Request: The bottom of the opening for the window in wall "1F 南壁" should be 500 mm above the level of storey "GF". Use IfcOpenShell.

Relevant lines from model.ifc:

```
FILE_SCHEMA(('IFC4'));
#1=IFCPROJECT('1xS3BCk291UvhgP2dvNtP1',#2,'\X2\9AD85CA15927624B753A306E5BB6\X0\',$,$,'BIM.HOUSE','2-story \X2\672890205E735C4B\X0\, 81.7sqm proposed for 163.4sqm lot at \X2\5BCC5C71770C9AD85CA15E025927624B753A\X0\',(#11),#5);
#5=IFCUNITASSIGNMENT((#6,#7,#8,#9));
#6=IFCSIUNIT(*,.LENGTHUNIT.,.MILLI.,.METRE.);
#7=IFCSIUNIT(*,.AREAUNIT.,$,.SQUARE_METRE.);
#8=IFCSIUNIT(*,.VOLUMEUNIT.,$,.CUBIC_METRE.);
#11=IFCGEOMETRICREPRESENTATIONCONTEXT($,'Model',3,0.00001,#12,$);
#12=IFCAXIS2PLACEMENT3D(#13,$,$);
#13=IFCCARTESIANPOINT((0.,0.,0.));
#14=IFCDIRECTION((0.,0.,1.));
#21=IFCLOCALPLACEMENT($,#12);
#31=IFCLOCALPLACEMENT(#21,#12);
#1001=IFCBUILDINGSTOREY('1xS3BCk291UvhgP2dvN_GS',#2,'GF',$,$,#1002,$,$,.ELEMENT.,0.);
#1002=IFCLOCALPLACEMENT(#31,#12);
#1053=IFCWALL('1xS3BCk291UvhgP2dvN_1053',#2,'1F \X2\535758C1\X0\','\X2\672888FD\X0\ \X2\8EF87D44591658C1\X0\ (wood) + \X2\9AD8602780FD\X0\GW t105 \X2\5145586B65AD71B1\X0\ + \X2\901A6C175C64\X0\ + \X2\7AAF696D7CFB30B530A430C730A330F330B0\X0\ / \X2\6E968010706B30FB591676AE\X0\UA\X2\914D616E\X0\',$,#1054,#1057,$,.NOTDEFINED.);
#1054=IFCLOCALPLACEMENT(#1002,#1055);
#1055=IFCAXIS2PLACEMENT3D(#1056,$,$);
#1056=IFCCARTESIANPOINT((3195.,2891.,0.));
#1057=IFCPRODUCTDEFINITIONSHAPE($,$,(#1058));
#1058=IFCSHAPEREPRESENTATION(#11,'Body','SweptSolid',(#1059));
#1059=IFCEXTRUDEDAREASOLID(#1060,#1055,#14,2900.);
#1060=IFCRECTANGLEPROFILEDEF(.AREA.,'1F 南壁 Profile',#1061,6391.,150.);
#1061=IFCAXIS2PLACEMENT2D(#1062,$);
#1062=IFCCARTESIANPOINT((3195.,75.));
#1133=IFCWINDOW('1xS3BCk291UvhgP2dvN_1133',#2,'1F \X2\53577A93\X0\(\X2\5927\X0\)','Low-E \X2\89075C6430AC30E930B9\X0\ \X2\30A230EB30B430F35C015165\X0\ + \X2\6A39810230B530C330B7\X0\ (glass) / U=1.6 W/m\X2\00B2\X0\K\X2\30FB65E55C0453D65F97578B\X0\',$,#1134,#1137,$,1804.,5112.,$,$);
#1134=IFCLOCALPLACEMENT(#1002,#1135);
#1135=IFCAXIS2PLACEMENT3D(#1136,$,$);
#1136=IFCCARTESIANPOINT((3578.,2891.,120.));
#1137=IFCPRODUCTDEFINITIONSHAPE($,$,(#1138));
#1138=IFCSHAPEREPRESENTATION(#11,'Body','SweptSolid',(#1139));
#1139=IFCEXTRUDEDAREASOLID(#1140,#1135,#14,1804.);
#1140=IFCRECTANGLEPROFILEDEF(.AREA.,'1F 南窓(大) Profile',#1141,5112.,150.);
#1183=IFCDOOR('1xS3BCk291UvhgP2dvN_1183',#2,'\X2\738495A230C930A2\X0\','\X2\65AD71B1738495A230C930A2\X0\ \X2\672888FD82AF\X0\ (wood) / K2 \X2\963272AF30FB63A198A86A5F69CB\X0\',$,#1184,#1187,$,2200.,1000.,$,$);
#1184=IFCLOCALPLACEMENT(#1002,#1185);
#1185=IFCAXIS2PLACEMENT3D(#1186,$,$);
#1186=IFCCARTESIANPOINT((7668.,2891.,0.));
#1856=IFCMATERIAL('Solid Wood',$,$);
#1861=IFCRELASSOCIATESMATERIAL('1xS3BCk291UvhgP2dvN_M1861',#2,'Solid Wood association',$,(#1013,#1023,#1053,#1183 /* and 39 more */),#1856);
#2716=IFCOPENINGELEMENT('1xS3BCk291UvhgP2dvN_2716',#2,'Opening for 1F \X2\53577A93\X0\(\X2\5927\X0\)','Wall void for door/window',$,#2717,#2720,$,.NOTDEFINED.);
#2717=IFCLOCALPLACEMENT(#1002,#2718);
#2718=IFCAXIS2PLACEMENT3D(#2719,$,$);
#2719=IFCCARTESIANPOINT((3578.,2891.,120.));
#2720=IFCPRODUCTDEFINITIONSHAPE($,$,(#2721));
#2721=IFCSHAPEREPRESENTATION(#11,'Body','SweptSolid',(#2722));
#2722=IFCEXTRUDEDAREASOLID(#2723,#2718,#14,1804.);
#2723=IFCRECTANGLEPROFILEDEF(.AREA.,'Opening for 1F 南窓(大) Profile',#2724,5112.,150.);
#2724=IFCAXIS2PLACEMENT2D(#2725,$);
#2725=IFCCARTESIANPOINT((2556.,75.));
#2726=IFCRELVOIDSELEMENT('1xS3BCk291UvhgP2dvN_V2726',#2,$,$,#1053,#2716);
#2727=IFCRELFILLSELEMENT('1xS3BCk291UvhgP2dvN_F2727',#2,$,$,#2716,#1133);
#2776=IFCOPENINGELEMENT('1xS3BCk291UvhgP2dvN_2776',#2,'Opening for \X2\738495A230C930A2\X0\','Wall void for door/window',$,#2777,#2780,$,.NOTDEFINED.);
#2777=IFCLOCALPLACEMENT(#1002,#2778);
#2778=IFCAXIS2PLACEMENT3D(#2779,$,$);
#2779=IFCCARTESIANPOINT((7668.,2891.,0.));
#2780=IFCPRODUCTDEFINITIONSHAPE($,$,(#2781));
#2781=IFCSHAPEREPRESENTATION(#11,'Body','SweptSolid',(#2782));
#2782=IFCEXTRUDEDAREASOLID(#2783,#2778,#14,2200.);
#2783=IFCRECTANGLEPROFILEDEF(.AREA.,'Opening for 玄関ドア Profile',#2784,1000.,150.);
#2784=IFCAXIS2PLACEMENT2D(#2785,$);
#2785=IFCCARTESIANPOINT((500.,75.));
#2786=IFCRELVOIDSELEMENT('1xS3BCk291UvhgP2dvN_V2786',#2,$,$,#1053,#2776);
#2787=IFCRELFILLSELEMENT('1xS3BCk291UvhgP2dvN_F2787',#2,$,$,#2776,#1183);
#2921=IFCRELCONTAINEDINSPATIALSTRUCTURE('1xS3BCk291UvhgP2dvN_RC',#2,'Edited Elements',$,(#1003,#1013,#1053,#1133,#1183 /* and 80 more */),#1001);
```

```python
import numpy as np
import ifcopenshell
import ifcopenshell.api.geometry
import ifcopenshell.geom
import ifcopenshell.util.element
import ifcopenshell.util.placement
import ifcopenshell.util.shape
import ifcopenshell.util.unit

model = ifcopenshell.open("model.ifc")
unit_scale = ifcopenshell.util.unit.calculate_unit_scale(model)

window = model.by_guid("1xS3BCk291UvhgP2dvN_1133")
opening = window.FillsVoids[0].RelatingOpeningElement
storey = ifcopenshell.util.element.get_container(window, ifc_class="IfcBuildingStorey")
level = ifcopenshell.util.placement.get_local_placement(storey.ObjectPlacement)[2, 3]

# The opening's origin need not be at the sill, so measure its lowest point.
shape = ifcopenshell.geom.create_shape(ifcopenshell.geom.settings(), opening)
bottom = ifcopenshell.util.shape.get_shape_bottom_elevation(shape, shape.geometry) / unit_scale
dz = level + 0.5 / unit_scale - bottom

shift = np.array([0.0, 0.0, dz])
# The window is not placed relative to its opening, so move both.
for product in (opening, window):
    matrix = ifcopenshell.util.placement.get_local_placement(product.ObjectPlacement)
    matrix[:3, 3] += shift
    ifcopenshell.api.geometry.edit_object_placement(model, product=product, matrix=matrix, is_si=False)

print(f"moved by {dz * unit_scale:+.3f} m")

model.write("model_rev.ifc")
```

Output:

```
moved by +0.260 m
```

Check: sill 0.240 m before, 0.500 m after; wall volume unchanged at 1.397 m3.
